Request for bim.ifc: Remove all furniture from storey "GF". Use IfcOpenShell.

First a look at what the model holds.

```python
import ifcopenshell
import ifcopenshell.util.element

model = ifcopenshell.open("bim.ifc")
print(model.schema)
storey = next(s for s in model.by_type("IfcBuildingStorey") if s.Name == "GF")
furniture = [e for e in ifcopenshell.util.element.get_decomposition(storey) if e.is_a("IfcFurnishingElement")]
seen = {}
for e in furniture:
    element_type = ifcopenshell.util.element.get_type(e)
    name = element_type.Name if element_type not in (None, e) else None
    seen[name] = seen.get(name, 0) + 1
for name, count in sorted(seen.items(), key=str):
    print(count, "x", name)
```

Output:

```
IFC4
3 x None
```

```python
import ifcopenshell
import ifcopenshell.api.root
import ifcopenshell.util.element

model = ifcopenshell.open("bim.ifc")

storey = next(s for s in model.by_type("IfcBuildingStorey") if s.Name == "GF")
furniture = [e for e in ifcopenshell.util.element.get_decomposition(storey) if e.is_a("IfcFurnishingElement")]

for e in furniture:
    ifcopenshell.api.root.remove_product(model, product=e)
print(len(furniture), "removed")

model.write("bim_v2.ifc")
```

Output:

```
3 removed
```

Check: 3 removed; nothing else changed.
